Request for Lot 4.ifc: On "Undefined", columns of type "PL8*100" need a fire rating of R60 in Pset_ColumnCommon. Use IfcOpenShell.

First a look at what the model holds.

```python
import ifcopenshell
import ifcopenshell.util.element

model = ifcopenshell.open("Lot 4.ifc")
print(model.schema)
storey = next(s for s in model.by_type("IfcBuildingStorey") if s.Name == "Undefined")
columns = [e for e in ifcopenshell.util.element.get_decomposition(storey) if e.is_a("IfcColumn")]
seen = {}
for e in columns:
    element_type = ifcopenshell.util.element.get_type(e)
    key = (element_type.Name if element_type != e and element_type else None, ifcopenshell.util.element.get_pset(e, "Pset_ColumnCommon", "FireRating"))
    seen[key] = seen.get(key, 0) + 1
for (name, value), count in sorted(seen.items(), key=str):
    print(count, "x", name, "|", value)
```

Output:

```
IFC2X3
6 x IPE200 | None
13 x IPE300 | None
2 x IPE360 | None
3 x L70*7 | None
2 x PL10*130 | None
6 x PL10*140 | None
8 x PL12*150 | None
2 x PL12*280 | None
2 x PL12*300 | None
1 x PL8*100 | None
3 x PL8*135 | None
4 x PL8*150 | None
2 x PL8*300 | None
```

```python
import ifcopenshell
import ifcopenshell.api.pset
import ifcopenshell.util.element

model = ifcopenshell.open("Lot 4.ifc")

storey = next(s for s in model.by_type("IfcBuildingStorey") if s.Name == "Undefined")
columns = [e for e in ifcopenshell.util.element.get_decomposition(storey) if e.is_a("IfcColumn")]

count = 0
for e in columns:
    element_type = ifcopenshell.util.element.get_type(e)
    if element_type in (None, e) or element_type.Name != "PL8*100":
        continue
    # add_pset returns the element's existing set when there is one.
    pset = ifcopenshell.api.pset.add_pset(model, product=e, name="Pset_ColumnCommon")
    ifcopenshell.api.pset.edit_pset(model, pset=pset, properties={"FireRating": "R60"})
    count += 1

print(count, "columns updated")

model.write("Lot 4_edited.ifc")
```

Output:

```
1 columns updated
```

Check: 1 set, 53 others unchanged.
